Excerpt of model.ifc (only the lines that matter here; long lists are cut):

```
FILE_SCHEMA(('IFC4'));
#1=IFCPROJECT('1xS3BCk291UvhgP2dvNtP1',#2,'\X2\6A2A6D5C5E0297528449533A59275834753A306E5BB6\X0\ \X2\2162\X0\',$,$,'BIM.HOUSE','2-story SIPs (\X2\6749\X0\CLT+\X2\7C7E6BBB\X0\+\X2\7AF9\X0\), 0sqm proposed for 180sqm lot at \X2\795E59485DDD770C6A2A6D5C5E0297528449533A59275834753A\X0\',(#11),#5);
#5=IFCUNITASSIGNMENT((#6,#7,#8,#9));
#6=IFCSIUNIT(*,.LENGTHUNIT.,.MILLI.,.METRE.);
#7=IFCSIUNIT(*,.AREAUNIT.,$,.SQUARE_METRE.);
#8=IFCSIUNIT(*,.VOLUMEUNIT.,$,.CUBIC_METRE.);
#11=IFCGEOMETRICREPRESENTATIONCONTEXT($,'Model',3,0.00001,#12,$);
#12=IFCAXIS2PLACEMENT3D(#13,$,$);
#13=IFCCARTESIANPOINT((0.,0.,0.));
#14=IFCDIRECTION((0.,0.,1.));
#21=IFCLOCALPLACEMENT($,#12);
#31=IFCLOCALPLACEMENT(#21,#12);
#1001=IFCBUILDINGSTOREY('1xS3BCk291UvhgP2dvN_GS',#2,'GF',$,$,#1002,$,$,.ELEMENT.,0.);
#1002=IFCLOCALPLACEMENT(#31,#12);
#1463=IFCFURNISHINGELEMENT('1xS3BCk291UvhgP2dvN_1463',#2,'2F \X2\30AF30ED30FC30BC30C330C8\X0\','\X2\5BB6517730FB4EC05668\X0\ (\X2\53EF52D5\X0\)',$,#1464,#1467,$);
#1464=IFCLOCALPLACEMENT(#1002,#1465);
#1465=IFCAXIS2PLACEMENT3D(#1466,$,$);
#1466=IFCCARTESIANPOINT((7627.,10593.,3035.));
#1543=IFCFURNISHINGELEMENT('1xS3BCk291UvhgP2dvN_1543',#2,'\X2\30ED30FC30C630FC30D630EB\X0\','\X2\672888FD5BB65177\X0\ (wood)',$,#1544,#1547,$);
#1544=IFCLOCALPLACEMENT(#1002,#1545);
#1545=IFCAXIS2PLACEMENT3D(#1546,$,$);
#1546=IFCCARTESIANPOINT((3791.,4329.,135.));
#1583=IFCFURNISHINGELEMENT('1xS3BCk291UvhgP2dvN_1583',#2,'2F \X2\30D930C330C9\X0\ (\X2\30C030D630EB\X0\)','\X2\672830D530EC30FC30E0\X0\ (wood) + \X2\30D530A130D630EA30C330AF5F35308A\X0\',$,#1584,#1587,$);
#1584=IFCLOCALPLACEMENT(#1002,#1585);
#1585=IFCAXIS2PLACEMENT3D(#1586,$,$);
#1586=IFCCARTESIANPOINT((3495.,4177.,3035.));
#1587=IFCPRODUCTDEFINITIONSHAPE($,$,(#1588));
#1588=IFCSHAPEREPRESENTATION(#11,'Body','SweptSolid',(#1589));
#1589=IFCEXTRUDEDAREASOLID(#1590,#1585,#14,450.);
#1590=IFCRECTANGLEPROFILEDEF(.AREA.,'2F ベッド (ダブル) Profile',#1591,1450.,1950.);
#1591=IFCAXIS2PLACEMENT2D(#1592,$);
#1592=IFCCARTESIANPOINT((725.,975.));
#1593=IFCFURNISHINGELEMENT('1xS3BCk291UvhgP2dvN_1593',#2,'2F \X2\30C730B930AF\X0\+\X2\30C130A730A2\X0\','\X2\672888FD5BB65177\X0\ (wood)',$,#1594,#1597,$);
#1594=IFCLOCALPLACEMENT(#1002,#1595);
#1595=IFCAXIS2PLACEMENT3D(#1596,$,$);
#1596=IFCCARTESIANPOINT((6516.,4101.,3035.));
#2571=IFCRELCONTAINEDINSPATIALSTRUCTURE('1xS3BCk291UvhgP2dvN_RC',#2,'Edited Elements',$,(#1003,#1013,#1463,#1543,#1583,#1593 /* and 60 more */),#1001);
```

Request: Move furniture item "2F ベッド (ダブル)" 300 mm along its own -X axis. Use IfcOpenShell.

```python
import ifcopenshell
import ifcopenshell.api.geometry
import ifcopenshell.util.placement
import ifcopenshell.util.unit

model = ifcopenshell.open("model.ifc")
unit_scale = ifcopenshell.util.unit.calculate_unit_scale(model)

item = model.by_guid("1xS3BCk291UvhgP2dvN_1583")
matrix = ifcopenshell.util.placement.get_local_placement(item.ObjectPlacement)
matrix[:3, 3] -= matrix[:3, 0] * 0.3 / unit_scale
ifcopenshell.api.geometry.edit_object_placement(model, product=item, matrix=matrix, is_si=False)

print(ifcopenshell.util.placement.get_local_placement(item.ObjectPlacement).round(3) + 0.0)

model.write("model_updated.ifc")
```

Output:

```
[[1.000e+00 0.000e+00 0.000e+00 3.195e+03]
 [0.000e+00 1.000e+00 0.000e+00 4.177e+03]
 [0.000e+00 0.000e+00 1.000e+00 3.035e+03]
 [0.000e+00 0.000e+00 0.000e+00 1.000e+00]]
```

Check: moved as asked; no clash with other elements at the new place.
